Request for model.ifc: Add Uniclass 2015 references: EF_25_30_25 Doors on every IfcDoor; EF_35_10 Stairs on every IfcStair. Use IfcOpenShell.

First a look at what the model holds.

```python
import ifcopenshell

model = ifcopenshell.open("model.ifc")
print(model.schema)
print("classifications:", [c.Name for c in model.by_type("IfcClassification")])
for ifc_class in ("IfcDoor", "IfcRoof", "IfcStair", "IfcWall", "IfcWindow"):
    print(ifc_class, len(model.by_type(ifc_class)))
```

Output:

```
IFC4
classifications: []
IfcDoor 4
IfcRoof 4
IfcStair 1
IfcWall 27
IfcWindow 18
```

```python
import ifcopenshell
import ifcopenshell.api.classification

model = ifcopenshell.open("model.ifc")

system = ifcopenshell.api.classification.add_classification(model, classification="Uniclass 2015")

codes = {
    "IfcDoor": ("EF_25_30_25", "Doors"),
    "IfcStair": ("EF_35_10", "Stairs"),
}
for ifc_class, (code, name) in codes.items():
    products = model.by_type(ifc_class)
    ifcopenshell.api.classification.add_reference(
        model, products=products, classification=system, identification=code, name=name
    )
    print(code, len(products))

model.write("model-out.ifc")
```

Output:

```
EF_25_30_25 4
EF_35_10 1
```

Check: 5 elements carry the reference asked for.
